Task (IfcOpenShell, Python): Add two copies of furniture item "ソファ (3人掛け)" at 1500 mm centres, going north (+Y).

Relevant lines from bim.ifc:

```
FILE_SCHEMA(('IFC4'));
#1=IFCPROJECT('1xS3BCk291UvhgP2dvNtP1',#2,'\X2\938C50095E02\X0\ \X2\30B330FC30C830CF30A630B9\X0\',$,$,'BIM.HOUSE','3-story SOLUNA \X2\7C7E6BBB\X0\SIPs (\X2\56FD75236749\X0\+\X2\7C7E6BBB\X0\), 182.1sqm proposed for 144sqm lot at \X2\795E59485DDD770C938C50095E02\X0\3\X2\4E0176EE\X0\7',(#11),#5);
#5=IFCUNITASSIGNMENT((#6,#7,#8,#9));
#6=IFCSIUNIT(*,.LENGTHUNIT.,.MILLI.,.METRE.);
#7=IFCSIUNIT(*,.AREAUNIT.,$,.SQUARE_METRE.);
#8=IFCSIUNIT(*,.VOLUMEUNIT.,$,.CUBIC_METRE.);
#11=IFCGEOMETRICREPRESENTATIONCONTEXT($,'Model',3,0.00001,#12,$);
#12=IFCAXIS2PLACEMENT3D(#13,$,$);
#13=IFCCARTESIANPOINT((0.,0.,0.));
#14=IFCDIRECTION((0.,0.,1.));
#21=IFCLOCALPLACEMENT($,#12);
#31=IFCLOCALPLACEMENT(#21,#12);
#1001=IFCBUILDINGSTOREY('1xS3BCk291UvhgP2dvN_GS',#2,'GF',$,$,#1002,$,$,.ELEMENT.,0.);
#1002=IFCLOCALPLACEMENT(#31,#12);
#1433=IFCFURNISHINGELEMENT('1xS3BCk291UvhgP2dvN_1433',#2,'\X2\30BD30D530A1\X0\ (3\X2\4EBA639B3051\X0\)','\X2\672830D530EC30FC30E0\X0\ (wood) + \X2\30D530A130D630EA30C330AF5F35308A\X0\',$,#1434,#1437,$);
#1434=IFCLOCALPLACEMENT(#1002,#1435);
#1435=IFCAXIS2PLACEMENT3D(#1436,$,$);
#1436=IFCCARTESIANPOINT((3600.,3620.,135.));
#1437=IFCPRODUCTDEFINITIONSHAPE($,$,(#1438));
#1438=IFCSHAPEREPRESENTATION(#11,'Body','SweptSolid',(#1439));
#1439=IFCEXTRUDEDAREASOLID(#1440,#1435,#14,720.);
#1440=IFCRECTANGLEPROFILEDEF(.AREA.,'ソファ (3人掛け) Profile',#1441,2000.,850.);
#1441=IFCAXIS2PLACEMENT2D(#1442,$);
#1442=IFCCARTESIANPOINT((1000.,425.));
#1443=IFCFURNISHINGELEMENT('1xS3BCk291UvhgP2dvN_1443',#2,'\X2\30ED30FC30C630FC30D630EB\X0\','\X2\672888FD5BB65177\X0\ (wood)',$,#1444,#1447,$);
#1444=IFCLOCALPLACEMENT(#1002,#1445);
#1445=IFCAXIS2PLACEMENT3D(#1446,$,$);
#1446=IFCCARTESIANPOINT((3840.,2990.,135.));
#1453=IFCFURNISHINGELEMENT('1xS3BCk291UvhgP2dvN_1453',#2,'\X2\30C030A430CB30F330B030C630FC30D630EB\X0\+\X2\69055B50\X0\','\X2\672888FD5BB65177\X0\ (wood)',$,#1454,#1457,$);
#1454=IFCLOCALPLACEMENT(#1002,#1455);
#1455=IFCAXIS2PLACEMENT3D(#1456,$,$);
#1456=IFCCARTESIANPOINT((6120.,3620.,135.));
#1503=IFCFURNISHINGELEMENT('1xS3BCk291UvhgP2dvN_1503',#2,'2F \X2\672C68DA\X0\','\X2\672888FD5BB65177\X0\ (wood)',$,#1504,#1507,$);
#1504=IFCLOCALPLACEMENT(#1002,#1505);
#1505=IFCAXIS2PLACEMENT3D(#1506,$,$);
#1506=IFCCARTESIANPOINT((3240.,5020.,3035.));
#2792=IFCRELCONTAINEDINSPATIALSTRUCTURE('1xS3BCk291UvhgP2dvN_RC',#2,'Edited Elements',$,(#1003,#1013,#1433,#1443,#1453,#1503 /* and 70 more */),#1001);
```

```python
import numpy as np
import ifcopenshell
import ifcopenshell.api.geometry
import ifcopenshell.api.root
import ifcopenshell.util.element
import ifcopenshell.util.placement

model = ifcopenshell.open("bim.ifc")


def reuse_history(source, copy):
    """copy_class also copies each property set's owner history, people and application; keep the originals."""
    for rel in copy.IsDefinedBy:
        if rel.is_a("IfcRelDefinesByProperties") and (history := rel.RelatingPropertyDefinition.OwnerHistory):
            rel.RelatingPropertyDefinition.OwnerHistory = source.OwnerHistory
            ifcopenshell.util.element.remove_deep2(model, history)


source = model.by_guid("1xS3BCk291UvhgP2dvN_1433")
base = ifcopenshell.util.placement.get_local_placement(source.ObjectPlacement)
step = np.array([0.0, 1.0, 0.0]) * 1500.0

for i in range(1, 3):
    copy = ifcopenshell.api.root.copy_class(model, product=source)
    copy.Representation = ifcopenshell.util.element.copy_deep(
        model, source.Representation, exclude=["IfcGeometricRepresentationContext", "IfcRepresentationMap"]
    )
    reuse_history(source, copy)
    matrix = base.copy()
    matrix[:3, 3] += i * step
    print("added at", matrix[:3, 3].round(3) + 0.0)
    ifcopenshell.api.geometry.edit_object_placement(model, product=copy, matrix=matrix, is_si=False)

model.write("bim-out.ifc")
```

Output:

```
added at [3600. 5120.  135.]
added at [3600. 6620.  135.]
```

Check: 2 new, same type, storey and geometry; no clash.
